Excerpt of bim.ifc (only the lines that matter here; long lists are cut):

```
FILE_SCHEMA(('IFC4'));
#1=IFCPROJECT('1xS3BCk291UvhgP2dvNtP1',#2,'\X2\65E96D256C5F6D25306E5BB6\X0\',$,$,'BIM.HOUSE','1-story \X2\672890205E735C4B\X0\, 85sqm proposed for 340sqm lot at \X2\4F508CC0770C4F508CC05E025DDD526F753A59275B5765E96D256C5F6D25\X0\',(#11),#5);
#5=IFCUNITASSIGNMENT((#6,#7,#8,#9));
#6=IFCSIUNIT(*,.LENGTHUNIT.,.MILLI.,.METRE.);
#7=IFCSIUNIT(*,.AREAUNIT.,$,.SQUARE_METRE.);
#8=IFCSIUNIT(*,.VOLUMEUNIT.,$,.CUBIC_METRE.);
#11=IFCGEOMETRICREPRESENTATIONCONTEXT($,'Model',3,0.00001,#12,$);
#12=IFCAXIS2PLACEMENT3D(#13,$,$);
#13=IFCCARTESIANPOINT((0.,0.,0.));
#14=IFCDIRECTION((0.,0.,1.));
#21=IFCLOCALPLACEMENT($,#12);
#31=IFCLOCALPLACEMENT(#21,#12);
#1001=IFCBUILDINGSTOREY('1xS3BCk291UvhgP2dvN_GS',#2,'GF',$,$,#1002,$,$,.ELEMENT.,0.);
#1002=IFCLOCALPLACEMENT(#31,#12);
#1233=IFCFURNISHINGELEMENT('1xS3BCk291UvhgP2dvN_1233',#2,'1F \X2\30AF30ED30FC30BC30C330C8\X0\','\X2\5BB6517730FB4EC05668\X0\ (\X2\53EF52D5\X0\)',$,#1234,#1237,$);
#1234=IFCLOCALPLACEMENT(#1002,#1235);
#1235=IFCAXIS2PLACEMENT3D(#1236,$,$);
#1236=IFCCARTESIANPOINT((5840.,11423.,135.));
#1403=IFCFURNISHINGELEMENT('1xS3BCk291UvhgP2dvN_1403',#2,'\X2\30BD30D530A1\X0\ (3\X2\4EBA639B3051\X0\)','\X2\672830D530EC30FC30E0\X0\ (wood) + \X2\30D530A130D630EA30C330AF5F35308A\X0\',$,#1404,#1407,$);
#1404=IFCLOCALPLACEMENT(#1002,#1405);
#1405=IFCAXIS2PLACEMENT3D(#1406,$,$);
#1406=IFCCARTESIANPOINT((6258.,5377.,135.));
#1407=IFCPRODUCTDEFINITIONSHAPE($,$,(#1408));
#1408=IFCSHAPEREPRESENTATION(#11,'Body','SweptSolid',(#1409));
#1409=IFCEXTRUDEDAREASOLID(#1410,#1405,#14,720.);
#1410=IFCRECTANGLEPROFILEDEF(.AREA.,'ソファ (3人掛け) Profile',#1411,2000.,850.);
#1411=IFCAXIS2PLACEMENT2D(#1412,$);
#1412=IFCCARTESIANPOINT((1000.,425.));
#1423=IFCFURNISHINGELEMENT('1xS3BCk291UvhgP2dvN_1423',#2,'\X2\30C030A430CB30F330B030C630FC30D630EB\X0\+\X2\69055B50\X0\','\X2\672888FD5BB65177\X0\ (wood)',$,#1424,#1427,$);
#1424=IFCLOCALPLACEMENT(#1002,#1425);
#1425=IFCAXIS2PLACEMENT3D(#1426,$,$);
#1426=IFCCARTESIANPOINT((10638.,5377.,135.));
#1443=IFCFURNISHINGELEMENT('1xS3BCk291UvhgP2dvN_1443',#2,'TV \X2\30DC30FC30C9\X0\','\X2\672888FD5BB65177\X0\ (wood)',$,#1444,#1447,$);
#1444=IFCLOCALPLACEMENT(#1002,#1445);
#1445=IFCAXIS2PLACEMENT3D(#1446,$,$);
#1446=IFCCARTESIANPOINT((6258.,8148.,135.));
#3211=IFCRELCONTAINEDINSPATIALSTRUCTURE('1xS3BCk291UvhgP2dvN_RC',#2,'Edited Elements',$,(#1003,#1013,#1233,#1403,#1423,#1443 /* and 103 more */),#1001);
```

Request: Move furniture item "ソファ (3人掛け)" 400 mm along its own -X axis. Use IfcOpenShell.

```python
import ifcopenshell
import ifcopenshell.api.geometry
import ifcopenshell.util.placement
import ifcopenshell.util.unit

model = ifcopenshell.open("bim.ifc")
unit_scale = ifcopenshell.util.unit.calculate_unit_scale(model)

item = model.by_id(1403)
matrix = ifcopenshell.util.placement.get_local_placement(item.ObjectPlacement)
matrix[:3, 3] -= matrix[:3, 0] * 0.4 / unit_scale
ifcopenshell.api.geometry.edit_object_placement(model, product=item, matrix=matrix, is_si=False)

print(ifcopenshell.util.placement.get_local_placement(item.ObjectPlacement).round(3) + 0.0)

model.write("bim_edited.ifc")
```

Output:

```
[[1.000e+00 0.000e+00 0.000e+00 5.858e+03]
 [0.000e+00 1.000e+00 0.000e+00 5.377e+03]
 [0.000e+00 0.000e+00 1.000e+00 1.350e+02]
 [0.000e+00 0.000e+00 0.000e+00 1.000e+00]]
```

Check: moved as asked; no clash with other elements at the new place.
